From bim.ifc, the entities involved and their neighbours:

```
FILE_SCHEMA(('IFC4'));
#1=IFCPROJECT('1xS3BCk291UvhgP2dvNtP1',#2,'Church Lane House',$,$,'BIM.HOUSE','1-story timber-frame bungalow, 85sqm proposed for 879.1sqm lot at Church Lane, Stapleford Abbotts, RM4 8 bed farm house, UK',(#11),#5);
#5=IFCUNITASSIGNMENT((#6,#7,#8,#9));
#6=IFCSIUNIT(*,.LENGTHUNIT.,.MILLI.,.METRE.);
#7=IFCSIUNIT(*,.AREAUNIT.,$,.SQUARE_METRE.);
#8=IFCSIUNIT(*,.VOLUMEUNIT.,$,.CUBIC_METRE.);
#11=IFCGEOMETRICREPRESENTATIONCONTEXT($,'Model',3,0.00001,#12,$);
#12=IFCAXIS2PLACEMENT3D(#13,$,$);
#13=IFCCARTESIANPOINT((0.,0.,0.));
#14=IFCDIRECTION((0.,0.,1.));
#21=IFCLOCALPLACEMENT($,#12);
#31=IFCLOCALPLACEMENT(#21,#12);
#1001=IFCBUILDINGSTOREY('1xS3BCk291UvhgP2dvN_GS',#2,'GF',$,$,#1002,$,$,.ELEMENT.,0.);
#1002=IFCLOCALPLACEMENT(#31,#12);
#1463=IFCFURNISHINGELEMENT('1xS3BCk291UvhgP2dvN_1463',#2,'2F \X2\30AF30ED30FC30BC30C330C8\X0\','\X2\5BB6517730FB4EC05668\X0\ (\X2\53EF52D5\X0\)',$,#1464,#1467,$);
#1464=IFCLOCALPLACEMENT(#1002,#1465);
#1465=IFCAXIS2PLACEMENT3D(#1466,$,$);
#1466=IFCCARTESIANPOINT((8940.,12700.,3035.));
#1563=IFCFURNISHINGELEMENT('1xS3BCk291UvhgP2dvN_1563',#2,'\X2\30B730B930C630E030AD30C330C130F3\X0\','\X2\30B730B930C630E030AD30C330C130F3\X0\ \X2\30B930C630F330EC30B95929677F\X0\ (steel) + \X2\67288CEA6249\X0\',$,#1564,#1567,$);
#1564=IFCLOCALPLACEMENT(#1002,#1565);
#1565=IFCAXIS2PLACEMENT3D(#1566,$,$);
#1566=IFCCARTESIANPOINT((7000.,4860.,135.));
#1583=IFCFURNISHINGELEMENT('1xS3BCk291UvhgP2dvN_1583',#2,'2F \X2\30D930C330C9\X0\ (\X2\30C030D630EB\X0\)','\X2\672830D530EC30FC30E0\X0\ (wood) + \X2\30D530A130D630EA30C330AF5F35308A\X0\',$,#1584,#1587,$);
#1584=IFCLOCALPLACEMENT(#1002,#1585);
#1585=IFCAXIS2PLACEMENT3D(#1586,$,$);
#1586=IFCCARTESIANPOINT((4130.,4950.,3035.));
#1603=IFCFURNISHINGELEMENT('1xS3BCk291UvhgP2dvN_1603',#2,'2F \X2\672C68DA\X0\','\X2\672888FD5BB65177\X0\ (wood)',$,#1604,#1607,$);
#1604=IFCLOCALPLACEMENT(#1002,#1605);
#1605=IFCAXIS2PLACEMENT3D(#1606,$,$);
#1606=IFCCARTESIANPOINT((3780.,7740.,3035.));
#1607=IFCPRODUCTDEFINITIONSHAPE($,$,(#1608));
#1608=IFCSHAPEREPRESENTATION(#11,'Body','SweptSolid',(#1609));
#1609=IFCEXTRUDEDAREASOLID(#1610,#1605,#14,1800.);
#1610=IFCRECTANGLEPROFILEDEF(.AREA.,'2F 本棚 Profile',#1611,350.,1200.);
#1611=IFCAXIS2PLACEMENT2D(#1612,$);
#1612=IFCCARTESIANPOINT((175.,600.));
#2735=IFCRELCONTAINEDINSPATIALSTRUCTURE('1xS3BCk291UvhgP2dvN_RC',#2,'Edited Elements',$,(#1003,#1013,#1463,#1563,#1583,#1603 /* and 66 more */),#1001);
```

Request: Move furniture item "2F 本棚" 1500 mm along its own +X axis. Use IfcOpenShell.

```python
import ifcopenshell
import ifcopenshell.api.geometry
import ifcopenshell.util.placement
import ifcopenshell.util.unit

model = ifcopenshell.open("bim.ifc")
unit_scale = ifcopenshell.util.unit.calculate_unit_scale(model)

item = model.by_guid("1xS3BCk291UvhgP2dvN_1603")
matrix = ifcopenshell.util.placement.get_local_placement(item.ObjectPlacement)
matrix[:3, 3] += matrix[:3, 0] * 1.5 / unit_scale
ifcopenshell.api.geometry.edit_object_placement(model, product=item, matrix=matrix, is_si=False)

print(ifcopenshell.util.placement.get_local_placement(item.ObjectPlacement).round(3) + 0.0)

model.write("bim-out.ifc")
```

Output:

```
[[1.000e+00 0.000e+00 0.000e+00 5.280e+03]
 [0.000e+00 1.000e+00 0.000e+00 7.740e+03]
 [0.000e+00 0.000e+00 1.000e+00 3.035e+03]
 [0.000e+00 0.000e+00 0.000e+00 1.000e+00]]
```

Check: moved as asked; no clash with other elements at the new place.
